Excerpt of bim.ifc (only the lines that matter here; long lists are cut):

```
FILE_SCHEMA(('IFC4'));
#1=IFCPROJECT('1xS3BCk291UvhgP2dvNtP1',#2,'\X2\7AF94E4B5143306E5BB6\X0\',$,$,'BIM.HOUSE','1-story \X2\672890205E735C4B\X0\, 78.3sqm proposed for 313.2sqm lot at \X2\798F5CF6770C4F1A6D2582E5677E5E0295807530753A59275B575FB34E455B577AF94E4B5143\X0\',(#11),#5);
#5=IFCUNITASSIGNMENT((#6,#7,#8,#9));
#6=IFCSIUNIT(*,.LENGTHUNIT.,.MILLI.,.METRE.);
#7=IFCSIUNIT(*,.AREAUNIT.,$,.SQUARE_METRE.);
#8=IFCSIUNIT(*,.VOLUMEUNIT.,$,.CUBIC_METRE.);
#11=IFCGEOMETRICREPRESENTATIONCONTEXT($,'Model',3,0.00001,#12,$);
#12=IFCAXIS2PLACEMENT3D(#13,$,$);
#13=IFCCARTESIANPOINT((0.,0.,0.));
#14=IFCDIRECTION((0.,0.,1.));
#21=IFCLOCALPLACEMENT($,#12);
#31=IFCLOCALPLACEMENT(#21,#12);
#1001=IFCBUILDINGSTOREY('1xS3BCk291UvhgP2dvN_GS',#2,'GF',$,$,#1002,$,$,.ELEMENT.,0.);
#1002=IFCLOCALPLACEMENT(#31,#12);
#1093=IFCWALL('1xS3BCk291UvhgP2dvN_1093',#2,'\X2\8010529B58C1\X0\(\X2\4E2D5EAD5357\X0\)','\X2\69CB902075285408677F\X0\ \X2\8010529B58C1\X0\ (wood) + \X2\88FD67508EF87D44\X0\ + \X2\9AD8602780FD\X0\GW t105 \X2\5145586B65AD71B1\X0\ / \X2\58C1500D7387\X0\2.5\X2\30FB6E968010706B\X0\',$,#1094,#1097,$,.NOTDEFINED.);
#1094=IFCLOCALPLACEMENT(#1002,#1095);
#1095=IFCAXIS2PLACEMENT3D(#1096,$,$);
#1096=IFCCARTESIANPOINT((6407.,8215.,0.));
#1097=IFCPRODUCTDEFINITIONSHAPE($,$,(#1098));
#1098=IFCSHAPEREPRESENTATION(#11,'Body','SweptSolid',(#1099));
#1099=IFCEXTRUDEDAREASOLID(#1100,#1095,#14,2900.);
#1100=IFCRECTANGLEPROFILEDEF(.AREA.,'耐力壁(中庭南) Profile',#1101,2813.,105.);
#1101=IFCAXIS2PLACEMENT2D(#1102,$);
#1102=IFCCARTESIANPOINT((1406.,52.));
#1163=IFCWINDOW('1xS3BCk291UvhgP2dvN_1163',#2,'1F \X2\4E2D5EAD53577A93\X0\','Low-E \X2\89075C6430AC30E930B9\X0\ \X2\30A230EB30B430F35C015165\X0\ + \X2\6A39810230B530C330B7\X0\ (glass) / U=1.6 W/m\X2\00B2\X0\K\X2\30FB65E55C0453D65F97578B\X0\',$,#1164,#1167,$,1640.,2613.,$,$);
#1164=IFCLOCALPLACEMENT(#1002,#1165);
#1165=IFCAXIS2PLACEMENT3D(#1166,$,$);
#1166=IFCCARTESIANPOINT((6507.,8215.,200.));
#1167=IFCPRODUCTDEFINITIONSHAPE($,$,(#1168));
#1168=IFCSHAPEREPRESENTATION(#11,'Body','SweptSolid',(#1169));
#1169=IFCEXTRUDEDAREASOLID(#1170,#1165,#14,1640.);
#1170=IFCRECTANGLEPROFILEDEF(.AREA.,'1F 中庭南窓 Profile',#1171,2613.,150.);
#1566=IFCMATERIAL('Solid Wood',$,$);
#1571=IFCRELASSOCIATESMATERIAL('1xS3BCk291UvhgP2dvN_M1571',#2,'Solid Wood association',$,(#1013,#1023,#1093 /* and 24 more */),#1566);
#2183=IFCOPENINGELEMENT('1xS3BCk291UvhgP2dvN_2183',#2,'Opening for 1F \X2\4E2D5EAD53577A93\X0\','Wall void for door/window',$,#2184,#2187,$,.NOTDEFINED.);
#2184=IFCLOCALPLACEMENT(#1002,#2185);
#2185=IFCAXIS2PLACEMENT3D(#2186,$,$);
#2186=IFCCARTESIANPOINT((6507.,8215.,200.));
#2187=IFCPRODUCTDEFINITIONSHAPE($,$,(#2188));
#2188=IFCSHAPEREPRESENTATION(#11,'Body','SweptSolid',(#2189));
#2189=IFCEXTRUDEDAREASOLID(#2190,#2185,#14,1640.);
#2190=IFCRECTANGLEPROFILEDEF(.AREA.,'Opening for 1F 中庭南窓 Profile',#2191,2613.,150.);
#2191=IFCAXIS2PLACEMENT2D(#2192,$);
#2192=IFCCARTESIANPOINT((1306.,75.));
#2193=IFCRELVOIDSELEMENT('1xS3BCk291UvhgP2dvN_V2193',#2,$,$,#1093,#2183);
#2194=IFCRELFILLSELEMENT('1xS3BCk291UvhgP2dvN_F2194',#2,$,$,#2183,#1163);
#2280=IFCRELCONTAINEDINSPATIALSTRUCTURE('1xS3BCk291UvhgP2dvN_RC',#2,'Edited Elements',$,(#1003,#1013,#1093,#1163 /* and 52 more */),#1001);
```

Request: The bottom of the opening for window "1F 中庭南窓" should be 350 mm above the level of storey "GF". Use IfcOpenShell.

```python
import numpy as np
import ifcopenshell
import ifcopenshell.api.geometry
import ifcopenshell.geom
import ifcopenshell.util.element
import ifcopenshell.util.placement
import ifcopenshell.util.shape
import ifcopenshell.util.unit

model = ifcopenshell.open("bim.ifc")
unit_scale = ifcopenshell.util.unit.calculate_unit_scale(model)

window = model.by_guid("1xS3BCk291UvhgP2dvN_1163")
opening = window.FillsVoids[0].RelatingOpeningElement
storey = ifcopenshell.util.element.get_container(window, ifc_class="IfcBuildingStorey")
level = ifcopenshell.util.placement.get_local_placement(storey.ObjectPlacement)[2, 3]

# The opening's origin need not be at the sill, so measure its lowest point.
shape = ifcopenshell.geom.create_shape(ifcopenshell.geom.settings(), opening)
bottom = ifcopenshell.util.shape.get_shape_bottom_elevation(shape, shape.geometry) / unit_scale
dz = level + 0.35 / unit_scale - bottom

shift = np.array([0.0, 0.0, dz])
# The window is not placed relative to its opening, so move both.
for product in (opening, window):
    matrix = ifcopenshell.util.placement.get_local_placement(product.ObjectPlacement)
    matrix[:3, 3] += shift
    ifcopenshell.api.geometry.edit_object_placement(model, product=product, matrix=matrix, is_si=False)

print(f"moved by {dz * unit_scale:+.3f} m")

model.write("bim-out.ifc")
```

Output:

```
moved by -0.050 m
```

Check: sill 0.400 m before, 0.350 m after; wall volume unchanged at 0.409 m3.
